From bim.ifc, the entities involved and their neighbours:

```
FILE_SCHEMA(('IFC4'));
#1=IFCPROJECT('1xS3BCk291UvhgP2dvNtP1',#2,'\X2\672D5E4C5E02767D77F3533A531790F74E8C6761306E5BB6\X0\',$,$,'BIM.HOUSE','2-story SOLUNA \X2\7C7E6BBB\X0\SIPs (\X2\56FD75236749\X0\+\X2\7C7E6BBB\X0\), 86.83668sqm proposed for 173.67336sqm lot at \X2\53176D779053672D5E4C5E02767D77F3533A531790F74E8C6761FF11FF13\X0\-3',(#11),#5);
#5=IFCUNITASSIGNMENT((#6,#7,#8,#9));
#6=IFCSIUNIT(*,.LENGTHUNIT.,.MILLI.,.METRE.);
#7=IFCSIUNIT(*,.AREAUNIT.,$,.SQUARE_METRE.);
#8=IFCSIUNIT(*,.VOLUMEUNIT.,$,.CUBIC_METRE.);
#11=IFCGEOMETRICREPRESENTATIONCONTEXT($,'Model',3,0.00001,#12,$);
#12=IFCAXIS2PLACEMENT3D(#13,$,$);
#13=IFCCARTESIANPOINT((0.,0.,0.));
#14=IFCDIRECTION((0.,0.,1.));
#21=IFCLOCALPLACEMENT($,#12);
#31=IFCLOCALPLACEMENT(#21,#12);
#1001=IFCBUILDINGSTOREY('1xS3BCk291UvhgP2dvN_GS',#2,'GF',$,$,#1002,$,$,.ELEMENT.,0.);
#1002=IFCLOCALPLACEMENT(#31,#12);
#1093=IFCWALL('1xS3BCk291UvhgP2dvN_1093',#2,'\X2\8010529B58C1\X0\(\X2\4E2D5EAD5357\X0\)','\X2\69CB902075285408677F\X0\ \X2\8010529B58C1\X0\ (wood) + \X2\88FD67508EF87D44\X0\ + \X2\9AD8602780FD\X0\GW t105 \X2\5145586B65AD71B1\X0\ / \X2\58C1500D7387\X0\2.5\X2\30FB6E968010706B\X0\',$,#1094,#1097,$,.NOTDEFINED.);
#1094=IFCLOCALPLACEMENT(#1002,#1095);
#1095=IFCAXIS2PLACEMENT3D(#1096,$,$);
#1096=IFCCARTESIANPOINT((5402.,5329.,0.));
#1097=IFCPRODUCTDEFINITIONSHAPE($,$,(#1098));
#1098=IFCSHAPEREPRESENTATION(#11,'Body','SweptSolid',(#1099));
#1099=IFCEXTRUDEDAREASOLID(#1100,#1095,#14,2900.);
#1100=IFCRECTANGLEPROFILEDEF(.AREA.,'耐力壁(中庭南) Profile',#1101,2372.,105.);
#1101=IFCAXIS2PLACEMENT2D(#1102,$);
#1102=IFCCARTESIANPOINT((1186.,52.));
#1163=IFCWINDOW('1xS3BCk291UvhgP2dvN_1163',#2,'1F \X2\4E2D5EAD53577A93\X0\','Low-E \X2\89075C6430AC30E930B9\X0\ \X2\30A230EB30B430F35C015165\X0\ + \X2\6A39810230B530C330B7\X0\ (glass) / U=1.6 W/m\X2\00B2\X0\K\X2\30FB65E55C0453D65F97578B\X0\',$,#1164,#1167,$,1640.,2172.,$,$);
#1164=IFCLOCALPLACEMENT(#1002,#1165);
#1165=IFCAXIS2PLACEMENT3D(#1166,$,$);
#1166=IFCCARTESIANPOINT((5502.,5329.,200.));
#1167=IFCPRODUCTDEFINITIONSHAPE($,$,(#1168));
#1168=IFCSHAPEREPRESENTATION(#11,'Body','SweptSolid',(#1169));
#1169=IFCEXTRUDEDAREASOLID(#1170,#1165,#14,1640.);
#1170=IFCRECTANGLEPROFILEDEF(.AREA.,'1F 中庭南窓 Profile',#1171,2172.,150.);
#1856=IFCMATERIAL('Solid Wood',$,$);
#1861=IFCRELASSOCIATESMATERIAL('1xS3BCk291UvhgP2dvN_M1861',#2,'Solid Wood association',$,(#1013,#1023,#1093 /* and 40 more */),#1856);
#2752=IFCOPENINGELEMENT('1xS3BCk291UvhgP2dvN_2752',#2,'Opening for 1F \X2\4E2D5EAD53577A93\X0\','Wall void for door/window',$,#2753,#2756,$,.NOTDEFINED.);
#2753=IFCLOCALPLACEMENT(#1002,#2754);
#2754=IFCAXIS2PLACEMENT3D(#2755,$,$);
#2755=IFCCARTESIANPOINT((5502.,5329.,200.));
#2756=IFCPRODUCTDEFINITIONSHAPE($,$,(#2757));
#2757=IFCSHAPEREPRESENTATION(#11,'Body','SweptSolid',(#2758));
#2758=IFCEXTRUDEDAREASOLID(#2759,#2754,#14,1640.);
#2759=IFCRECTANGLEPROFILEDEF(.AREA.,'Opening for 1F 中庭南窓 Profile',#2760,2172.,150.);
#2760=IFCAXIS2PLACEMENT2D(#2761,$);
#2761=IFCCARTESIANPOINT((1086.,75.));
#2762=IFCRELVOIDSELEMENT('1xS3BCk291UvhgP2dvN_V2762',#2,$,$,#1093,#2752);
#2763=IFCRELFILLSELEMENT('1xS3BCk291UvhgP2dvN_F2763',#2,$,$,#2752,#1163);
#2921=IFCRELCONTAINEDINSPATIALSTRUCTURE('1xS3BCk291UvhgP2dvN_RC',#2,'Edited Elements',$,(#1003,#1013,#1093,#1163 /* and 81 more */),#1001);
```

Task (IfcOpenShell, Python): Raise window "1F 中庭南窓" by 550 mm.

```python
import numpy as np
import ifcopenshell
import ifcopenshell.api.geometry
import ifcopenshell.util.placement
import ifcopenshell.util.unit

model = ifcopenshell.open("bim.ifc")
unit_scale = ifcopenshell.util.unit.calculate_unit_scale(model)

window = model.by_guid("1xS3BCk291UvhgP2dvN_1163")
opening = window.FillsVoids[0].RelatingOpeningElement
dz = 0.55 / unit_scale

shift = np.array([0.0, 0.0, dz])
# The window is not placed relative to its opening, so move both.
for product in (opening, window):
    matrix = ifcopenshell.util.placement.get_local_placement(product.ObjectPlacement)
    matrix[:3, 3] += shift
    ifcopenshell.api.geometry.edit_object_placement(model, product=product, matrix=matrix, is_si=False)

print(f"moved by {dz * unit_scale:+.3f} m")

model.write("bim_edited.ifc")
```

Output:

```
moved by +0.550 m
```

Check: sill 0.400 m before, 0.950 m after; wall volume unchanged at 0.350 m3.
